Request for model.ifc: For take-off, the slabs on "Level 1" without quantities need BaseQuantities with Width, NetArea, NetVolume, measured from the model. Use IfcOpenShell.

First a look at what the model holds.

```python
import ifcopenshell
import ifcopenshell.util.element
import ifcopenshell.util.unit

model = ifcopenshell.open("model.ifc")
print(model.schema)
for unit_type in ("LENGTHUNIT", "AREAUNIT", "VOLUMEUNIT"):
    print(unit_type, ifcopenshell.util.unit.calculate_unit_scale(model, unit_type))
storey = next(s for s in model.by_type("IfcBuildingStorey") if s.Name == "Level 1")
slabs = [e for e in ifcopenshell.util.element.get_decomposition(storey) if e.is_a("IfcSlab")]
for e in sorted(slabs, key=lambda e: e.id()):
    print(e.id(), e.is_a(), e.Name, list(ifcopenshell.util.element.get_psets(e, qtos_only=True)), sep=" | ")
```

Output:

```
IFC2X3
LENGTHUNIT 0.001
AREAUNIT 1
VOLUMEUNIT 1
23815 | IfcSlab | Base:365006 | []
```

```python
import ifcopenshell
import ifcopenshell.api.pset
import ifcopenshell.geom
import ifcopenshell.util.element
import ifcopenshell.util.shape
import ifcopenshell.util.unit

model = ifcopenshell.open("model.ifc")
unit_scale = ifcopenshell.util.unit.calculate_unit_scale(model)
area_scale = ifcopenshell.util.unit.calculate_unit_scale(model, "AREAUNIT")
volume_scale = ifcopenshell.util.unit.calculate_unit_scale(model, "VOLUMEUNIT")
settings = ifcopenshell.geom.settings()

storey = next(s for s in model.by_type("IfcBuildingStorey") if s.Name == "Level 1")
slabs = [e for e in ifcopenshell.util.element.get_decomposition(storey) if e.is_a("IfcSlab")]

for e in sorted(slabs, key=lambda e: e.id()):
    if ifcopenshell.util.element.get_psets(e, qtos_only=True, should_inherit=False):
        continue
    # Geometry comes back in metres, in the element's own axes.
    shape = ifcopenshell.geom.create_shape(settings, e)
    values = {
        "Width": ifcopenshell.util.shape.get_z(shape.geometry) / unit_scale,
        "NetArea": ifcopenshell.util.shape.get_footprint_area(shape.geometry) / area_scale,
        "NetVolume": ifcopenshell.util.shape.get_volume(shape.geometry) / volume_scale,
    }
    qto = ifcopenshell.api.pset.add_qto(model, product=e, name="BaseQuantities")
    ifcopenshell.api.pset.edit_qto(model, qto=qto, properties=values)
    print(e.id(), {k: round(v, 3) for k, v in values.items()})

model.write("model_rev.ifc")
```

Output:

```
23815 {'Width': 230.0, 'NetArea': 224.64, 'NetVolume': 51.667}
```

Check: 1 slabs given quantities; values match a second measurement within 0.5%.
